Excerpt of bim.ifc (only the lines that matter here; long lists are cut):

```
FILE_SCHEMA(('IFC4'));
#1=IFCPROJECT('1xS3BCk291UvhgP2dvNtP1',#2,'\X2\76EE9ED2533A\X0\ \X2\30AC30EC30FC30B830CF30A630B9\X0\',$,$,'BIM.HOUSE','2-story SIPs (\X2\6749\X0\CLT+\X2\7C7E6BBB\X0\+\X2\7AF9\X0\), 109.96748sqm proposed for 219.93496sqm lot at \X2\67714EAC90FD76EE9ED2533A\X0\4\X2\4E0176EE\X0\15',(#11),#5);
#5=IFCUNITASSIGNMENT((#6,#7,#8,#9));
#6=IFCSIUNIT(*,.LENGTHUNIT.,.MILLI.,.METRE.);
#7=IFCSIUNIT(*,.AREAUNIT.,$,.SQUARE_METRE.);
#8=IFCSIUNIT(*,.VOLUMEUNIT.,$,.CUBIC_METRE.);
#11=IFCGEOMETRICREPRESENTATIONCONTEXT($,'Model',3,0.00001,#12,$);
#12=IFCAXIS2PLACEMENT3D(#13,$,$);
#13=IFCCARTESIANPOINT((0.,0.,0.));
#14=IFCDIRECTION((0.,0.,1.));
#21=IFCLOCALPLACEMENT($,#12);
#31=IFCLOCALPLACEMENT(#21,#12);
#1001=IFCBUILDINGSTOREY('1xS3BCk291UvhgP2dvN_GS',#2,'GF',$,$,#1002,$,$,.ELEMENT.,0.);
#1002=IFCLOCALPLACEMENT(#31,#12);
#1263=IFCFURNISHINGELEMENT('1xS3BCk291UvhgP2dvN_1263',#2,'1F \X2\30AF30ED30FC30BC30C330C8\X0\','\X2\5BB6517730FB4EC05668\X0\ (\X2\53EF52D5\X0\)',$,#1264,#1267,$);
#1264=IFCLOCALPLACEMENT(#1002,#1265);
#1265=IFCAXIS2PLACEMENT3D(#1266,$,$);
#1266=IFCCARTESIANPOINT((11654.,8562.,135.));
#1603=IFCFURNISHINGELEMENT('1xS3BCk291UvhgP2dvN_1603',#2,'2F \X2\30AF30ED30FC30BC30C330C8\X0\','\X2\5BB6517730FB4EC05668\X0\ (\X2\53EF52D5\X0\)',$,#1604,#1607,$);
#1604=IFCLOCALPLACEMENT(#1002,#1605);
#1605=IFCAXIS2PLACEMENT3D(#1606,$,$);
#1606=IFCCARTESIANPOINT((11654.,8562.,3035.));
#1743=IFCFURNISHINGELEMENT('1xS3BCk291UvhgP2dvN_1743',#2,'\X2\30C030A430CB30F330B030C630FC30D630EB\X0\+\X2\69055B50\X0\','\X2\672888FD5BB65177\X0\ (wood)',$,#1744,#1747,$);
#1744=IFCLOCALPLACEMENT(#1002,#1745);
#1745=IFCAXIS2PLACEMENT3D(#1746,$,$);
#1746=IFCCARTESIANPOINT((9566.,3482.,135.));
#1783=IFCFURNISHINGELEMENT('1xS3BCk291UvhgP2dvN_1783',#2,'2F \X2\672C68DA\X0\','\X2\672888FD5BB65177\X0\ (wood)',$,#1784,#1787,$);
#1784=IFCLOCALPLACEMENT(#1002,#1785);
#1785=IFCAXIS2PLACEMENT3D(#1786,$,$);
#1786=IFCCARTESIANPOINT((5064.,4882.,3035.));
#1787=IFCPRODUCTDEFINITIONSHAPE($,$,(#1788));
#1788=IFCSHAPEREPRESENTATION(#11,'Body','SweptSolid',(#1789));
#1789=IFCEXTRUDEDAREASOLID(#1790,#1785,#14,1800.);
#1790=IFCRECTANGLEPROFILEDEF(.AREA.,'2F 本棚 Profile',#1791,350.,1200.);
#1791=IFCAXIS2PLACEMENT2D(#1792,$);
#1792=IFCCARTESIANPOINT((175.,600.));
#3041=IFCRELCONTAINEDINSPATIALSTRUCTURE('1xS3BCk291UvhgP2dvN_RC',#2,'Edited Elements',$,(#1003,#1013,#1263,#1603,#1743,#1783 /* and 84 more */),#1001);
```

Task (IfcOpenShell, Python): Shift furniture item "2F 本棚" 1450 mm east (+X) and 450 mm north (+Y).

```python
import ifcopenshell
import ifcopenshell.api.geometry
import ifcopenshell.util.placement
import ifcopenshell.util.unit

model = ifcopenshell.open("bim.ifc")
unit_scale = ifcopenshell.util.unit.calculate_unit_scale(model)

item = model.by_guid("1xS3BCk291UvhgP2dvN_1783")
matrix = ifcopenshell.util.placement.get_local_placement(item.ObjectPlacement)
matrix[0, 3] += 1.45 / unit_scale
matrix[1, 3] += 0.45 / unit_scale
ifcopenshell.api.geometry.edit_object_placement(model, product=item, matrix=matrix, is_si=False)

print(ifcopenshell.util.placement.get_local_placement(item.ObjectPlacement).round(3) + 0.0)

model.write("bim-out.ifc")
```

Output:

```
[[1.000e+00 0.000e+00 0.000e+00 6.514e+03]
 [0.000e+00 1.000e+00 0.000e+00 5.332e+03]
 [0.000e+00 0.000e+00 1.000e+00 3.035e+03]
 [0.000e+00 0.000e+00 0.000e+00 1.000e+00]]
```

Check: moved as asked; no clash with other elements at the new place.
